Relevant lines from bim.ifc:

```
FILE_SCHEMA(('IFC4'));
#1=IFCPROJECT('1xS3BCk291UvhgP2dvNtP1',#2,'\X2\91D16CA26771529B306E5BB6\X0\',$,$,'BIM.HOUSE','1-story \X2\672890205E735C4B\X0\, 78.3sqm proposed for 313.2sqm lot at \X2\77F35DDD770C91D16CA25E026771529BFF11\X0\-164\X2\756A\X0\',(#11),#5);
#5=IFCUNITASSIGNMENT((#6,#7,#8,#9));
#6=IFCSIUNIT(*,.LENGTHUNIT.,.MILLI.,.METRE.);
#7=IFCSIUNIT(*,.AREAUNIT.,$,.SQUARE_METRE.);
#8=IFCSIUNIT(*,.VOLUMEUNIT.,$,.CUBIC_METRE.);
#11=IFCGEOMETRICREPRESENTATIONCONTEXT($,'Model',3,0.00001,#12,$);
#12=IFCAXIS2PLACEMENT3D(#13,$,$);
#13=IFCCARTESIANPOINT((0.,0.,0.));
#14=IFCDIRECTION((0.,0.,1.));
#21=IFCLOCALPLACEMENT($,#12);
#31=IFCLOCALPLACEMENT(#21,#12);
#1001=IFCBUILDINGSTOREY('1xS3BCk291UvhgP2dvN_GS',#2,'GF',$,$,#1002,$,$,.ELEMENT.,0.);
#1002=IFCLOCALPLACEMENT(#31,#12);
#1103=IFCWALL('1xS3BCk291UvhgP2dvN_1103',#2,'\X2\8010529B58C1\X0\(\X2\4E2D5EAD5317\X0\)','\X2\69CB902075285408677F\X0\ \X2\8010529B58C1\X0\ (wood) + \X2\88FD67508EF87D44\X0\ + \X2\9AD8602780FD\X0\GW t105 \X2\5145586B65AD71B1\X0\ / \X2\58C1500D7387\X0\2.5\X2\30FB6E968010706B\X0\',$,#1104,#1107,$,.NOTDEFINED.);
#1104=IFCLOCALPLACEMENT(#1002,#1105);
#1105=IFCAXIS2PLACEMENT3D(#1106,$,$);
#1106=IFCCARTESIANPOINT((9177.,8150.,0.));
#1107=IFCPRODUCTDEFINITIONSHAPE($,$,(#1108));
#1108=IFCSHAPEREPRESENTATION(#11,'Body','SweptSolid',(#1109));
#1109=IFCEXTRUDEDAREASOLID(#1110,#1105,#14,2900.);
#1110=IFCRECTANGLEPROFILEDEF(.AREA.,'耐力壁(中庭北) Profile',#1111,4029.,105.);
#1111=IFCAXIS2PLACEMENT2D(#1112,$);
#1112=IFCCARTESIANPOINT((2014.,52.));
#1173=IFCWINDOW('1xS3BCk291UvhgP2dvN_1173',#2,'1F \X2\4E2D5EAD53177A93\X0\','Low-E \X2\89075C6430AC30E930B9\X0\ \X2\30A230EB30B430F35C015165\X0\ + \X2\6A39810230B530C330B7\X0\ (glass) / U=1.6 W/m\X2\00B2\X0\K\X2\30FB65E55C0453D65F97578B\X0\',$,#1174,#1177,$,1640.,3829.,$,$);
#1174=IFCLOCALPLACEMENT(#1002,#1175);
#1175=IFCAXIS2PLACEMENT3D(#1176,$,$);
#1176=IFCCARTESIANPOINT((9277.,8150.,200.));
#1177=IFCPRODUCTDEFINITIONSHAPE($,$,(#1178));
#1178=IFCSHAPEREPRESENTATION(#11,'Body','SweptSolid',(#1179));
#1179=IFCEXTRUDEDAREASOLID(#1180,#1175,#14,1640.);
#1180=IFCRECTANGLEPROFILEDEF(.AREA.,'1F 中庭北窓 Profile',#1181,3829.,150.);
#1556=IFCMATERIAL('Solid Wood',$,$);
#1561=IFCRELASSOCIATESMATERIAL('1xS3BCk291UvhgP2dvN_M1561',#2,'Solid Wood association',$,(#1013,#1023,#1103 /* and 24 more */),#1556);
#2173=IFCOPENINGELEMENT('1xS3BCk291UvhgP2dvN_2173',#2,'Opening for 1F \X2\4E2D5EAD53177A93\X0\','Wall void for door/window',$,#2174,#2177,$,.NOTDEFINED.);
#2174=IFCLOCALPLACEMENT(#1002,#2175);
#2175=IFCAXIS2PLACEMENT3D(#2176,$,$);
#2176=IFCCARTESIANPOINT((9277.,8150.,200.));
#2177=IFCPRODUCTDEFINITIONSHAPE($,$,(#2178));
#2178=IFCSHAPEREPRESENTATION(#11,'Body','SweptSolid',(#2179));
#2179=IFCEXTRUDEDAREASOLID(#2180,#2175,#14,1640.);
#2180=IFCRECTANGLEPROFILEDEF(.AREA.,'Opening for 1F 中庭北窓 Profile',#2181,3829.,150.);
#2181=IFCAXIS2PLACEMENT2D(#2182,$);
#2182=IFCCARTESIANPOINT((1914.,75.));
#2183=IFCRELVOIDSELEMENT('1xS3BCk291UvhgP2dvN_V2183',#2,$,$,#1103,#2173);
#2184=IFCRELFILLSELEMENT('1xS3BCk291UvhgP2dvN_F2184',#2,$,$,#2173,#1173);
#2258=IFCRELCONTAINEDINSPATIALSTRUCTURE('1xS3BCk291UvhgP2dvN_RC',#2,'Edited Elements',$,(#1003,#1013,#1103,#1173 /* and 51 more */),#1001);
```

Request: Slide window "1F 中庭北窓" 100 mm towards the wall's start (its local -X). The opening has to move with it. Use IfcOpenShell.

```python
import ifcopenshell
import ifcopenshell.api.geometry
import ifcopenshell.util.placement

model = ifcopenshell.open("bim.ifc")

window = model.by_id(1173)
opening = window.FillsVoids[0].RelatingOpeningElement
wall = opening.VoidsElements[0].RelatingBuildingElement

wall_matrix = ifcopenshell.util.placement.get_local_placement(wall.ObjectPlacement)
shift = wall_matrix[:3, 0] * -100.0
before = ifcopenshell.util.placement.get_local_placement(window.ObjectPlacement)[:3, 3].copy()

# The window is not placed relative to its opening, so move both.
for product in (opening, window):
    matrix = ifcopenshell.util.placement.get_local_placement(product.ObjectPlacement)
    matrix[:3, 3] += shift
    ifcopenshell.api.geometry.edit_object_placement(model, product=product, matrix=matrix, is_si=False)

after = ifcopenshell.util.placement.get_local_placement(window.ObjectPlacement)[:3, 3]
print("window moved by", (after - before).round(3) + 0.0)

model.write("bim-out.ifc")
```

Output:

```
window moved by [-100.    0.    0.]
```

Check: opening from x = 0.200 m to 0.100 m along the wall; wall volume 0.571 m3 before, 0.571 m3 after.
